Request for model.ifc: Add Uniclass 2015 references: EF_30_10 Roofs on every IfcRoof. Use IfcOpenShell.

First a look at what the model holds.

```python
import ifcopenshell

model = ifcopenshell.open("model.ifc")
print(model.schema)
print("classifications:", [c.Name for c in model.by_type("IfcClassification")])
for ifc_class in ("IfcDoor", "IfcRoof", "IfcStair", "IfcWall", "IfcWindow"):
    print(ifc_class, len(model.by_type(ifc_class)))
```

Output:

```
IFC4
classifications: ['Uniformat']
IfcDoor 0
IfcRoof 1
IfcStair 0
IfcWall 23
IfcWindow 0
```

```python
import ifcopenshell
import ifcopenshell.api.classification

model = ifcopenshell.open("model.ifc")

system = ifcopenshell.api.classification.add_classification(model, classification="Uniclass 2015")

codes = {
    "IfcRoof": ("EF_30_10", "Roofs"),
}
for ifc_class, (code, name) in codes.items():
    products = model.by_type(ifc_class)
    ifcopenshell.api.classification.add_reference(
        model, products=products, classification=system, identification=code, name=name
    )
    print(code, len(products))

model.write("model_rev.ifc")
```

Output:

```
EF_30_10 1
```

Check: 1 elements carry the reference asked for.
